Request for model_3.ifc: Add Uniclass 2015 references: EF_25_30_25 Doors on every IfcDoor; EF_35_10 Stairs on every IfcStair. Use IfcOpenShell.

First a look at what the model holds.

```python
import ifcopenshell

model = ifcopenshell.open("model_3.ifc")
print(model.schema)
print("classifications:", [c.Name for c in model.by_type("IfcClassification")])
for ifc_class in ("IfcDoor", "IfcRoof", "IfcStair", "IfcWall", "IfcWindow"):
    print(ifc_class, len(model.by_type(ifc_class)))
```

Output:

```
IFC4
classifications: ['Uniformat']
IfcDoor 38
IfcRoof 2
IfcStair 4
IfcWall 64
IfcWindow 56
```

```python
import ifcopenshell
import ifcopenshell.api.classification

model = ifcopenshell.open("model_3.ifc")

system = ifcopenshell.api.classification.add_classification(model, classification="Uniclass 2015")

codes = {
    "IfcDoor": ("EF_25_30_25", "Doors"),
    "IfcStair": ("EF_35_10", "Stairs"),
}
for ifc_class, (code, name) in codes.items():
    products = model.by_type(ifc_class)
    ifcopenshell.api.classification.add_reference(
        model, products=products, classification=system, identification=code, name=name
    )
    print(code, len(products))

model.write("model_3_edited.ifc")
```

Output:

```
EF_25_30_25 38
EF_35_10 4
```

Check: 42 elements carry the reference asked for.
